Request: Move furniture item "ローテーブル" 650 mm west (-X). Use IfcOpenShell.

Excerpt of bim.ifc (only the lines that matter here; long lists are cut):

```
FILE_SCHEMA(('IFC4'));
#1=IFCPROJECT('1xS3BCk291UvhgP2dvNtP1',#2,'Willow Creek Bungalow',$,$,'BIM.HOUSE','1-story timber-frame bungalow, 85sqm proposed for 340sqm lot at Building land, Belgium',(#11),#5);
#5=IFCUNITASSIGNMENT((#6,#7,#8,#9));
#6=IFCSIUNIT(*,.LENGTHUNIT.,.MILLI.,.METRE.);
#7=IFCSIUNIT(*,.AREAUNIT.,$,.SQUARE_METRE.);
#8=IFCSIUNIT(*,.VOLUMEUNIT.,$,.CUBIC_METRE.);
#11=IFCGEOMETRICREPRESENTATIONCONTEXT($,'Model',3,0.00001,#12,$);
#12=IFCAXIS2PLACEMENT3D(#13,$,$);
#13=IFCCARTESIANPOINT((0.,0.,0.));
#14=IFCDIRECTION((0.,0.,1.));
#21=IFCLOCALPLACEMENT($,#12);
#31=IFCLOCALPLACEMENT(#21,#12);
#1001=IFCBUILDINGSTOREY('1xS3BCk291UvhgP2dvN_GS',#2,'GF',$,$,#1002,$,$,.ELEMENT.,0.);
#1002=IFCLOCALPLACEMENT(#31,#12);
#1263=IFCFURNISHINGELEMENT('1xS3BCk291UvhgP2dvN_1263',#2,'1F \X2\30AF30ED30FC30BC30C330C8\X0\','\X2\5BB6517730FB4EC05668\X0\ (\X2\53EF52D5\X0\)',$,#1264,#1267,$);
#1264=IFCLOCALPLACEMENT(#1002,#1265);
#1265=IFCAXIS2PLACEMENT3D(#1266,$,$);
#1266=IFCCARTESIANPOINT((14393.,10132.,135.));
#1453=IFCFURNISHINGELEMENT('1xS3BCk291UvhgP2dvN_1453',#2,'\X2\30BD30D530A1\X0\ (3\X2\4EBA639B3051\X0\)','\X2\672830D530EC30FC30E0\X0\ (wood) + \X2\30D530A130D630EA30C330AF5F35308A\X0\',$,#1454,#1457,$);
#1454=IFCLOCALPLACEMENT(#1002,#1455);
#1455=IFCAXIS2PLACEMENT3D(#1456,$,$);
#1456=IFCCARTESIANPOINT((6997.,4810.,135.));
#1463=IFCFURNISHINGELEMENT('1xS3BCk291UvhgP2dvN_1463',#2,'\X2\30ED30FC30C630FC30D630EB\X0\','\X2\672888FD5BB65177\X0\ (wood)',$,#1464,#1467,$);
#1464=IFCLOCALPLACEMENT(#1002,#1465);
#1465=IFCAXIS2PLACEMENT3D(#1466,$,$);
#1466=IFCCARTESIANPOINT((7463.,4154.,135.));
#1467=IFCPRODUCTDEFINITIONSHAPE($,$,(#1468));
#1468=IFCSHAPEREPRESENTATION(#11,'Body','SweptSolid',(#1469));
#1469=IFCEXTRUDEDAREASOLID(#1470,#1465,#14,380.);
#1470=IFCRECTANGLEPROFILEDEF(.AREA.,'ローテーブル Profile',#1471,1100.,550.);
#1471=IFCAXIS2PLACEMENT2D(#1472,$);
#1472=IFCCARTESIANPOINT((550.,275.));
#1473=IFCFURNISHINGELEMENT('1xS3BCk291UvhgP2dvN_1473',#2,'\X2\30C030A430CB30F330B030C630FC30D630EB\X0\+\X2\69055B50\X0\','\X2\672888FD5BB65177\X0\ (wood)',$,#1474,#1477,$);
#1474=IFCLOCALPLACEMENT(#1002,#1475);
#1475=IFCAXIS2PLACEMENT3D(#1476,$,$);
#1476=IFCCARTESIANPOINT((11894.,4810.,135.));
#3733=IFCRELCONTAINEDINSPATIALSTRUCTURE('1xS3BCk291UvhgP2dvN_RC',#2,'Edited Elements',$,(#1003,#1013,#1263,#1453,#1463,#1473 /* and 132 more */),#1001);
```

```python
import ifcopenshell
import ifcopenshell.api.geometry
import ifcopenshell.util.placement
import ifcopenshell.util.unit

model = ifcopenshell.open("bim.ifc")
unit_scale = ifcopenshell.util.unit.calculate_unit_scale(model)

item = model.by_guid("1xS3BCk291UvhgP2dvN_1463")
matrix = ifcopenshell.util.placement.get_local_placement(item.ObjectPlacement)
matrix[0, 3] -= 0.65 / unit_scale
ifcopenshell.api.geometry.edit_object_placement(model, product=item, matrix=matrix, is_si=False)

print(ifcopenshell.util.placement.get_local_placement(item.ObjectPlacement).round(3) + 0.0)

model.write("bim_rev.ifc")
```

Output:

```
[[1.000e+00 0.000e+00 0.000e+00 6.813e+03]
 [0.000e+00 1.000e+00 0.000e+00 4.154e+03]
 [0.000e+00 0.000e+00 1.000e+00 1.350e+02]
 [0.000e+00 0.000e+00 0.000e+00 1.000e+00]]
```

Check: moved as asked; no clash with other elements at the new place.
